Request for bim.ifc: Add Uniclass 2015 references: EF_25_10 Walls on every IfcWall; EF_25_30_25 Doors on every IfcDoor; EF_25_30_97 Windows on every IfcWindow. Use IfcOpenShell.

First a look at what the model holds.

```python
import ifcopenshell

model = ifcopenshell.open("bim.ifc")
print(model.schema)
print("classifications:", [c.Name for c in model.by_type("IfcClassification")])
for ifc_class in ("IfcDoor", "IfcRoof", "IfcStair", "IfcWall", "IfcWindow"):
    print(ifc_class, len(model.by_type(ifc_class)))
```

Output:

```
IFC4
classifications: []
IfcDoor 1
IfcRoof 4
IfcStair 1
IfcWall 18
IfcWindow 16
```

```python
import ifcopenshell
import ifcopenshell.api.classification

model = ifcopenshell.open("bim.ifc")

system = ifcopenshell.api.classification.add_classification(model, classification="Uniclass 2015")

codes = {
    "IfcWall": ("EF_25_10", "Walls"),
    "IfcDoor": ("EF_25_30_25", "Doors"),
    "IfcWindow": ("EF_25_30_97", "Windows"),
}
for ifc_class, (code, name) in codes.items():
    products = model.by_type(ifc_class)
    ifcopenshell.api.classification.add_reference(
        model, products=products, classification=system, identification=code, name=name
    )
    print(code, len(products))

model.write("bim_rev.ifc")
```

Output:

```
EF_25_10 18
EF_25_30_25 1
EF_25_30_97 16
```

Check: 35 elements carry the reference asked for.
